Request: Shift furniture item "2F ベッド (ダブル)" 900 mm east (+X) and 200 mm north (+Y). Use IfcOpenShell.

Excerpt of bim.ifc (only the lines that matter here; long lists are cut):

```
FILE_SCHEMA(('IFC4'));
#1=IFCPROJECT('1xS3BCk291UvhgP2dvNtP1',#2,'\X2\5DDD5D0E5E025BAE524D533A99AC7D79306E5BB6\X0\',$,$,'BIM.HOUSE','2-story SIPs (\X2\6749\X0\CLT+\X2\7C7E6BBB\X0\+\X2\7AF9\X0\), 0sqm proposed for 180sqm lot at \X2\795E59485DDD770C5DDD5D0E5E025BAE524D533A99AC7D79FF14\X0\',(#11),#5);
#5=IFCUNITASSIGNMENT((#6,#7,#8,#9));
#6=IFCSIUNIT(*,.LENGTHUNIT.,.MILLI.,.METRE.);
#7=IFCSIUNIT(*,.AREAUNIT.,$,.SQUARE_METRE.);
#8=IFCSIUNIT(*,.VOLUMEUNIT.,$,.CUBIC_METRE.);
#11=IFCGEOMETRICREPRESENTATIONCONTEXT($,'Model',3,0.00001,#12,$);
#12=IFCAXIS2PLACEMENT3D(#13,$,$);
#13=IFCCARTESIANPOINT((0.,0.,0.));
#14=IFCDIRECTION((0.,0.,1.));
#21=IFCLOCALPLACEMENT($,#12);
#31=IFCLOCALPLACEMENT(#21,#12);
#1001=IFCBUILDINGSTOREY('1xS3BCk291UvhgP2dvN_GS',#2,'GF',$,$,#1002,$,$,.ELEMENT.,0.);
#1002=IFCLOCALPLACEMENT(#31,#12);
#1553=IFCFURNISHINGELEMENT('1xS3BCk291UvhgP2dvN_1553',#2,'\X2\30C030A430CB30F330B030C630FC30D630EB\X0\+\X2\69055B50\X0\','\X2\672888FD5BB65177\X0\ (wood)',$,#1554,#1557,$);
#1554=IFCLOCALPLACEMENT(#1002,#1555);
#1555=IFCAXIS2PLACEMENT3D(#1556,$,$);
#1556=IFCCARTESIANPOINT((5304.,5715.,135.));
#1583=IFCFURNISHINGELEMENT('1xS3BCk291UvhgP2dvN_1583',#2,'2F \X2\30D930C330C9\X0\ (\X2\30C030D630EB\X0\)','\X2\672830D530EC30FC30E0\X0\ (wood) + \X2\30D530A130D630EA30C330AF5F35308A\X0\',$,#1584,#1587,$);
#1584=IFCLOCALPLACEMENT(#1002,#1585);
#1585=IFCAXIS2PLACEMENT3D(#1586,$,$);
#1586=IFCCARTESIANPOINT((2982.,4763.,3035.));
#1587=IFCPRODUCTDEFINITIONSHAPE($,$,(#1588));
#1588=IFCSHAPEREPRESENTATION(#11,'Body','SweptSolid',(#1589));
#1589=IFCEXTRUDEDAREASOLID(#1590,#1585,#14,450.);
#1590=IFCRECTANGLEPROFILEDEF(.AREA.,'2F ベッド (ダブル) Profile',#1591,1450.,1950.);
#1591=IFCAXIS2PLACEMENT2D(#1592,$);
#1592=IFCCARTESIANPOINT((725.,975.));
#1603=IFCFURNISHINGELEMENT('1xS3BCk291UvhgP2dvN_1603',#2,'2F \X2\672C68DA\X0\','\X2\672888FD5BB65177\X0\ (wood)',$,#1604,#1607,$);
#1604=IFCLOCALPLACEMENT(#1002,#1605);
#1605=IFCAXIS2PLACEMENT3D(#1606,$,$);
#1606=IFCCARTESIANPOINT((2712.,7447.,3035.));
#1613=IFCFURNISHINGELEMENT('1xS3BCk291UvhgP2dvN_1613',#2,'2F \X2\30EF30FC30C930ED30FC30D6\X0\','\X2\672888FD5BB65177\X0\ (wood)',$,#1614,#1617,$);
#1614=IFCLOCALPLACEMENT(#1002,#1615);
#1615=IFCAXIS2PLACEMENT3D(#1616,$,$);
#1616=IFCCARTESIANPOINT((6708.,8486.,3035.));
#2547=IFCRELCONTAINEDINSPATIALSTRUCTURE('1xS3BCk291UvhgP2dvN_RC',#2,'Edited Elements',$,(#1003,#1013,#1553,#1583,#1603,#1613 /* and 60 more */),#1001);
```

```python
import ifcopenshell
import ifcopenshell.api.geometry
import ifcopenshell.util.placement
import ifcopenshell.util.unit

model = ifcopenshell.open("bim.ifc")
unit_scale = ifcopenshell.util.unit.calculate_unit_scale(model)

item = model.by_guid("1xS3BCk291UvhgP2dvN_1583")
matrix = ifcopenshell.util.placement.get_local_placement(item.ObjectPlacement)
matrix[0, 3] += 0.9 / unit_scale
matrix[1, 3] += 0.2 / unit_scale
ifcopenshell.api.geometry.edit_object_placement(model, product=item, matrix=matrix, is_si=False)

print(ifcopenshell.util.placement.get_local_placement(item.ObjectPlacement).round(3) + 0.0)

model.write("bim_edited.ifc")
```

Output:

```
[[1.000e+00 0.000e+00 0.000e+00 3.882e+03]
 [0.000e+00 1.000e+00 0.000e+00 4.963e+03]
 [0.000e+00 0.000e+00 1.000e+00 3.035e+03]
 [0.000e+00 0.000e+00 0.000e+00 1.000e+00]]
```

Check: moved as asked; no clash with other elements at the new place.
